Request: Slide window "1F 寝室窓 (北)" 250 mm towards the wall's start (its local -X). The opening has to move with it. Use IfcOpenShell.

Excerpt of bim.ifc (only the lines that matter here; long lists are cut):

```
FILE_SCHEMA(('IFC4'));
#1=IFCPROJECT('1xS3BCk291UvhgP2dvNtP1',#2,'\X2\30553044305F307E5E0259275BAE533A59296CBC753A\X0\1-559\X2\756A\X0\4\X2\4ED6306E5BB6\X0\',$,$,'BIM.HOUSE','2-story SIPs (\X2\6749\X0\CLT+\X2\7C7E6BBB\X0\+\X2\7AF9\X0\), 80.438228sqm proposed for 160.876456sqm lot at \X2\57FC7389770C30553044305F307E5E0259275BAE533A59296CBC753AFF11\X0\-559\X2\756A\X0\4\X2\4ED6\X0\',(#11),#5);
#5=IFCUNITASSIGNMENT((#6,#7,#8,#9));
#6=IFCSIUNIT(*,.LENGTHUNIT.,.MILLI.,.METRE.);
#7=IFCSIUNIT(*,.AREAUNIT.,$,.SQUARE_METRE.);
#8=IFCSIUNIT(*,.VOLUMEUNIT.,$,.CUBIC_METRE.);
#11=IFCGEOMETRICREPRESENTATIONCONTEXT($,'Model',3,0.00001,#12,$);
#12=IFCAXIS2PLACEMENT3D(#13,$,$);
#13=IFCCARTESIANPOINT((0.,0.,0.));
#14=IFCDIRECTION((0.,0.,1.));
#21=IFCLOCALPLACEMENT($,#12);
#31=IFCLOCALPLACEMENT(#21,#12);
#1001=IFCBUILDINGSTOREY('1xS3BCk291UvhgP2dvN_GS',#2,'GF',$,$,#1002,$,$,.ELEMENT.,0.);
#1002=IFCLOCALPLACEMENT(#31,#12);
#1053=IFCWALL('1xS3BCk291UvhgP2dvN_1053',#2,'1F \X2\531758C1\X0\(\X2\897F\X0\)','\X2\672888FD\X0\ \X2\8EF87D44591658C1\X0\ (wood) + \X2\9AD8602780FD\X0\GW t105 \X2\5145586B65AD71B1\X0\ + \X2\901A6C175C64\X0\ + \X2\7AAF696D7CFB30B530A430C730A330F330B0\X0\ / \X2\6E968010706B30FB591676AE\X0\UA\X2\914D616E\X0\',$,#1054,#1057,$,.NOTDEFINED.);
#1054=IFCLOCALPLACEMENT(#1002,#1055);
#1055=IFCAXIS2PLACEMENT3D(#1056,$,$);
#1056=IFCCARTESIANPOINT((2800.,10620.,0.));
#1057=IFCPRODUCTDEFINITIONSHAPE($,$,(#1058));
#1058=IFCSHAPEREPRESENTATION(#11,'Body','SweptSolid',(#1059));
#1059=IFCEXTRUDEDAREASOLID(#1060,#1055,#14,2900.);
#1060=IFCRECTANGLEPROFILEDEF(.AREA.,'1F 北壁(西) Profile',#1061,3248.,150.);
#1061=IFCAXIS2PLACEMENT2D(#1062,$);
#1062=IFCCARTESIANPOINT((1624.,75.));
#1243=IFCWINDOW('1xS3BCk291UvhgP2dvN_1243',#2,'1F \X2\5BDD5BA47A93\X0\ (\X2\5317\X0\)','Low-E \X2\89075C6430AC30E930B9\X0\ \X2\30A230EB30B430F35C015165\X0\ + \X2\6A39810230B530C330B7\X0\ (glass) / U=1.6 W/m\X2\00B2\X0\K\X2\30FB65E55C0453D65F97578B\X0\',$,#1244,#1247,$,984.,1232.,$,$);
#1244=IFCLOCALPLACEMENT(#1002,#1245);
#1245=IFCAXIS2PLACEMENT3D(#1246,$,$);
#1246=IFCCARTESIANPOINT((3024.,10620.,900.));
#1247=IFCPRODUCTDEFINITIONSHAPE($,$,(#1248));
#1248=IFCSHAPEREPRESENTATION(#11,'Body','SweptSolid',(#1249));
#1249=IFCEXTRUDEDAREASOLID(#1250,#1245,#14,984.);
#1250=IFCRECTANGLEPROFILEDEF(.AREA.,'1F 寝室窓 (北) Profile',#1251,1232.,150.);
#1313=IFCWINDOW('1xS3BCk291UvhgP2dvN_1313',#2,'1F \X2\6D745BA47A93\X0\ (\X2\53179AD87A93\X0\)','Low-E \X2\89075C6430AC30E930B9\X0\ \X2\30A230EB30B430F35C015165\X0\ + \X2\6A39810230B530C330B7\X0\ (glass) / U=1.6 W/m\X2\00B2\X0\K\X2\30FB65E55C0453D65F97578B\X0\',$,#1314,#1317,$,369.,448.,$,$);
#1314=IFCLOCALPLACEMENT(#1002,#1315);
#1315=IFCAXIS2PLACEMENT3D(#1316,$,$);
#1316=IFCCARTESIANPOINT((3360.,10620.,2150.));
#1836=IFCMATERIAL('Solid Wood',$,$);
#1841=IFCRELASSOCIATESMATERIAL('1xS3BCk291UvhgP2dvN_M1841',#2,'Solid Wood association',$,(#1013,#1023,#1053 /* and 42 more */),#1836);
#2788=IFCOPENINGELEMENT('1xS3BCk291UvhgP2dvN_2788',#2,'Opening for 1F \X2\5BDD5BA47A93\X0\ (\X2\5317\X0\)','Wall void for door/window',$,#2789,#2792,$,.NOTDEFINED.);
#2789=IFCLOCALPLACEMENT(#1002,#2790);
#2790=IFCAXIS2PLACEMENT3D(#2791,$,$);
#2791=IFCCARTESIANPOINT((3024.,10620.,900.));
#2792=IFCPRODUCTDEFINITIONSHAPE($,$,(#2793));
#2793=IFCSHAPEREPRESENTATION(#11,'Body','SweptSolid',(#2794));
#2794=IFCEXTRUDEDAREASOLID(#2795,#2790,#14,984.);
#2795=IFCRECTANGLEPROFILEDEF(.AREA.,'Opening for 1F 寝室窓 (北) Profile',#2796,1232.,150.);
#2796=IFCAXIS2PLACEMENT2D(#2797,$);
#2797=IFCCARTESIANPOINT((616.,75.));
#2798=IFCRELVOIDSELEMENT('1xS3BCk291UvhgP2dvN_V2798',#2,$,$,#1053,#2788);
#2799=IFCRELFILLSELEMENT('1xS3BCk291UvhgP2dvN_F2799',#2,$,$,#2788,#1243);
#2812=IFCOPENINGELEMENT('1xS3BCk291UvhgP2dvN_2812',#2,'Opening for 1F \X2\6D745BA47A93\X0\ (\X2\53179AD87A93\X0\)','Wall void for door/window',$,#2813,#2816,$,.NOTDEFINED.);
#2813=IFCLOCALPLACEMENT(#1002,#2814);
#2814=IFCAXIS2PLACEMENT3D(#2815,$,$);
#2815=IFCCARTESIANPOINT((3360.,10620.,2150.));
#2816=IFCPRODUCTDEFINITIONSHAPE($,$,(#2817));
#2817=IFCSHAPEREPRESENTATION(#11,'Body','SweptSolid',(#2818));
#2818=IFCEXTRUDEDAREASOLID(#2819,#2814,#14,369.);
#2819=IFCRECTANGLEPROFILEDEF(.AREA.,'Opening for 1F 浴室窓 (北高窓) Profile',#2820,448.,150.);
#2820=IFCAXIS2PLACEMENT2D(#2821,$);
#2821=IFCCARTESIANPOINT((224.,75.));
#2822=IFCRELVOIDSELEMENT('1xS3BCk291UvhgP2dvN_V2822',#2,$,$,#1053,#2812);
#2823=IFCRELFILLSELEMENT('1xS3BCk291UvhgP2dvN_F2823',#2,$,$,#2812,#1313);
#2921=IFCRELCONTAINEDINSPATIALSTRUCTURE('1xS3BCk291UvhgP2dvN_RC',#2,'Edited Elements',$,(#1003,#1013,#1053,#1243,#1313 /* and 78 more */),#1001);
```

```python
import ifcopenshell
import ifcopenshell.api.geometry
import ifcopenshell.util.placement
import ifcopenshell.util.unit

model = ifcopenshell.open("bim.ifc")
unit_scale = ifcopenshell.util.unit.calculate_unit_scale(model)

window = model.by_guid("1xS3BCk291UvhgP2dvN_1243")
opening = window.FillsVoids[0].RelatingOpeningElement
wall = opening.VoidsElements[0].RelatingBuildingElement

wall_matrix = ifcopenshell.util.placement.get_local_placement(wall.ObjectPlacement)
shift = wall_matrix[:3, 0] * -0.25 / unit_scale
before = ifcopenshell.util.placement.get_local_placement(window.ObjectPlacement)[:3, 3].copy()

# The window is not placed relative to its opening, so move both.
for product in (opening, window):
    matrix = ifcopenshell.util.placement.get_local_placement(product.ObjectPlacement)
    matrix[:3, 3] += shift
    ifcopenshell.api.geometry.edit_object_placement(model, product=product, matrix=matrix, is_si=False)

after = ifcopenshell.util.placement.get_local_placement(window.ObjectPlacement)[:3, 3]
print("window moved by", (after - before).round(3) + 0.0)

model.write("bim_updated.ifc")
```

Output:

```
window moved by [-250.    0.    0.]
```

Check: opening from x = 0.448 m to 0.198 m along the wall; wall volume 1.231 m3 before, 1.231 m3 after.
